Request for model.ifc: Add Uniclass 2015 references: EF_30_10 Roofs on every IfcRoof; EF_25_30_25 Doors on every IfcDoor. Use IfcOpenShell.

First a look at what the model holds.

```python
import ifcopenshell

model = ifcopenshell.open("model.ifc")
print(model.schema)
print("classifications:", [c.Name for c in model.by_type("IfcClassification")])
for ifc_class in ("IfcDoor", "IfcRoof", "IfcStair", "IfcWall", "IfcWindow"):
    print(ifc_class, len(model.by_type(ifc_class)))
```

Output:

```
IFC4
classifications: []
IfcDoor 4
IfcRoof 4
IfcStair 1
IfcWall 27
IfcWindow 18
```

```python
import ifcopenshell
import ifcopenshell.api.classification

model = ifcopenshell.open("model.ifc")

system = ifcopenshell.api.classification.add_classification(model, classification="Uniclass 2015")

codes = {
    "IfcRoof": ("EF_30_10", "Roofs"),
    "IfcDoor": ("EF_25_30_25", "Doors"),
}
for ifc_class, (code, name) in codes.items():
    products = model.by_type(ifc_class)
    ifcopenshell.api.classification.add_reference(
        model, products=products, classification=system, identification=code, name=name
    )
    print(code, len(products))

model.write("model_updated.ifc")
```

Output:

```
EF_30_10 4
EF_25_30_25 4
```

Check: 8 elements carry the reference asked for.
